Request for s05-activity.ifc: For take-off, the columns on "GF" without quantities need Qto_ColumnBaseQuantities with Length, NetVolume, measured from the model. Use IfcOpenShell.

First a look at what the model holds.

```python
import ifcopenshell
import ifcopenshell.util.element
import ifcopenshell.util.unit

model = ifcopenshell.open("s05-activity.ifc")
print(model.schema)
for unit_type in ("LENGTHUNIT", "AREAUNIT", "VOLUMEUNIT"):
    print(unit_type, ifcopenshell.util.unit.calculate_unit_scale(model, unit_type))
storey = next(s for s in model.by_type("IfcBuildingStorey") if s.Name == "GF")
columns = [e for e in ifcopenshell.util.element.get_decomposition(storey) if e.is_a("IfcColumn")]
for e in sorted(columns, key=lambda e: e.id()):
    print(e.id(), e.is_a(), e.Name, list(ifcopenshell.util.element.get_psets(e, qtos_only=True)), sep=" | ")
```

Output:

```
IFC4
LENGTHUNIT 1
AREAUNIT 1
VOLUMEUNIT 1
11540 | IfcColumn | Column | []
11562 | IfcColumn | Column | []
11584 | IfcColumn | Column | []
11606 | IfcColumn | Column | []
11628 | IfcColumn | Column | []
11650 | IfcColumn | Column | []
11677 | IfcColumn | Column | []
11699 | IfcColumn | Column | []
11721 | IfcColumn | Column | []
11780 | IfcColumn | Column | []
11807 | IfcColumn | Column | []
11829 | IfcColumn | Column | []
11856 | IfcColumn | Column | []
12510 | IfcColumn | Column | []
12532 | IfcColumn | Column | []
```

```python
import ifcopenshell
import ifcopenshell.api.pset
import ifcopenshell.geom
import ifcopenshell.util.element
import ifcopenshell.util.shape
import ifcopenshell.util.unit

model = ifcopenshell.open("s05-activity.ifc")
unit_scale = ifcopenshell.util.unit.calculate_unit_scale(model)
volume_scale = ifcopenshell.util.unit.calculate_unit_scale(model, "VOLUMEUNIT")
settings = ifcopenshell.geom.settings()

storey = next(s for s in model.by_type("IfcBuildingStorey") if s.Name == "GF")
columns = [e for e in ifcopenshell.util.element.get_decomposition(storey) if e.is_a("IfcColumn")]

for e in sorted(columns, key=lambda e: e.id()):
    if ifcopenshell.util.element.get_psets(e, qtos_only=True, should_inherit=False):
        continue
    # Geometry comes back in metres, in the element's own axes.
    shape = ifcopenshell.geom.create_shape(settings, e)
    values = {
        "Length": ifcopenshell.util.shape.get_z(shape.geometry) / unit_scale,
        "NetVolume": ifcopenshell.util.shape.get_volume(shape.geometry) / volume_scale,
    }
    qto = ifcopenshell.api.pset.add_qto(model, product=e, name="Qto_ColumnBaseQuantities")
    ifcopenshell.api.pset.edit_qto(model, qto=qto, properties=values)
    print(e.id(), {k: round(v, 3) for k, v in values.items()})

model.write("s05-activity_updated.ifc")
```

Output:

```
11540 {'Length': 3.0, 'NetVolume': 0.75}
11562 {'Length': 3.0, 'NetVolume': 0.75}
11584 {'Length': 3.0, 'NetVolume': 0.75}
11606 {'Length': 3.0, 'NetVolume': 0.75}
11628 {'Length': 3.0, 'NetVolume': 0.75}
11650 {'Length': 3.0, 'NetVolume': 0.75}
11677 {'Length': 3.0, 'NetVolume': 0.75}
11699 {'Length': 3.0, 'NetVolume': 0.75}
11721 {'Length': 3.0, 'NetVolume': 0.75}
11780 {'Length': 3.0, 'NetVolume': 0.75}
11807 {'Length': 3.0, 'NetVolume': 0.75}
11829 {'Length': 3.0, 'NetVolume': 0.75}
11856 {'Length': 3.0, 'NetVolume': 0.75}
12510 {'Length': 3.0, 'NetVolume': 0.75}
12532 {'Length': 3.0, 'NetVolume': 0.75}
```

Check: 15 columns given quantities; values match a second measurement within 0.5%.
